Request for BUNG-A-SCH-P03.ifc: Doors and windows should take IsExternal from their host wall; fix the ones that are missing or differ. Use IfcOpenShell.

First a look at what the model holds.

```python
import ifcopenshell
import ifcopenshell.util.element

model = ifcopenshell.open("BUNG-A-SCH-P03.ifc")
print(model.schema)
seen = {}
for e in model.by_type("IfcDoor") + model.by_type("IfcWindow"):
    if not e.FillsVoids:
        continue
    host = e.FillsVoids[0].RelatingOpeningElement.VoidsElements[0].RelatingBuildingElement
    own = ifcopenshell.util.element.get_pset(e, f"Pset_{e.is_a()[3:].removesuffix('StandardCase')}Common", "IsExternal")
    wall = ifcopenshell.util.element.get_pset(host, "Pset_WallCommon", "IsExternal")
    seen[e.is_a(), own, wall] = seen.get((e.is_a(), own, wall), 0) + 1
for (cls, own, wall), count in sorted(seen.items(), key=str):
    print(count, cls, "IsExternal:", own, "| host wall:", wall)
```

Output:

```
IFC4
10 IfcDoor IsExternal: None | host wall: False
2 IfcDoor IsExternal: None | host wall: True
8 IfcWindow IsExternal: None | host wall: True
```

```python
import ifcopenshell
import ifcopenshell.api.pset
import ifcopenshell.util.element

model = ifcopenshell.open("BUNG-A-SCH-P03.ifc")

count = 0
for ifc_class, pset_name in (("IfcDoor", "Pset_DoorCommon"), ("IfcWindow", "Pset_WindowCommon")):
    for e in model.by_type(ifc_class):
        if not e.FillsVoids:
            continue
        host = e.FillsVoids[0].RelatingOpeningElement.VoidsElements[0].RelatingBuildingElement
        external = ifcopenshell.util.element.get_pset(host, "Pset_WallCommon", "IsExternal")
        if external is None or ifcopenshell.util.element.get_pset(e, pset_name, "IsExternal") == external:
            continue
        pset = ifcopenshell.api.pset.add_pset(model, product=e, name=pset_name)
        ifcopenshell.api.pset.edit_pset(model, pset=pset, properties={"IsExternal": external})
        count += 1

print(count, "updated")

model.write("BUNG-A-SCH-P03_updated.ifc")
```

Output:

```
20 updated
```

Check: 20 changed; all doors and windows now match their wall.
